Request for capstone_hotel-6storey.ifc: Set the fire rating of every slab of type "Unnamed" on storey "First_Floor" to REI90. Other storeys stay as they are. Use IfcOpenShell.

First a look at what the model holds.

```python
import ifcopenshell
import ifcopenshell.util.element

model = ifcopenshell.open("capstone_hotel-6storey.ifc")
print(model.schema)
storey = next(s for s in model.by_type("IfcBuildingStorey") if s.Name == "First_Floor")
slabs = [e for e in ifcopenshell.util.element.get_decomposition(storey) if e.is_a("IfcSlab")]
seen = {}
for e in slabs:
    element_type = ifcopenshell.util.element.get_type(e)
    key = (element_type.Name if element_type != e and element_type else None, ifcopenshell.util.element.get_pset(e, "Pset_SlabCommon", "FireRating"))
    seen[key] = seen.get(key, 0) + 1
for (name, value), count in sorted(seen.items(), key=str):
    print(count, "x", name, "|", value)
```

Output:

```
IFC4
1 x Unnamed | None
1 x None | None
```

```python
import ifcopenshell
import ifcopenshell.api.pset
import ifcopenshell.util.element

model = ifcopenshell.open("capstone_hotel-6storey.ifc")

storey = next(s for s in model.by_type("IfcBuildingStorey") if s.Name == "First_Floor")
slabs = [e for e in ifcopenshell.util.element.get_decomposition(storey) if e.is_a("IfcSlab")]

count = 0
for e in slabs:
    element_type = ifcopenshell.util.element.get_type(e)
    if element_type in (None, e) or element_type.Name != "Unnamed":
        continue
    # add_pset returns the element's existing set when there is one.
    pset = ifcopenshell.api.pset.add_pset(model, product=e, name="Pset_SlabCommon")
    ifcopenshell.api.pset.edit_pset(model, pset=pset, properties={"FireRating": "REI90"})
    count += 1

print(count, "slabs updated")

model.write("capstone_hotel-6storey_v2.ifc")
```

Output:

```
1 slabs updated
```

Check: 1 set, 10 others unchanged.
